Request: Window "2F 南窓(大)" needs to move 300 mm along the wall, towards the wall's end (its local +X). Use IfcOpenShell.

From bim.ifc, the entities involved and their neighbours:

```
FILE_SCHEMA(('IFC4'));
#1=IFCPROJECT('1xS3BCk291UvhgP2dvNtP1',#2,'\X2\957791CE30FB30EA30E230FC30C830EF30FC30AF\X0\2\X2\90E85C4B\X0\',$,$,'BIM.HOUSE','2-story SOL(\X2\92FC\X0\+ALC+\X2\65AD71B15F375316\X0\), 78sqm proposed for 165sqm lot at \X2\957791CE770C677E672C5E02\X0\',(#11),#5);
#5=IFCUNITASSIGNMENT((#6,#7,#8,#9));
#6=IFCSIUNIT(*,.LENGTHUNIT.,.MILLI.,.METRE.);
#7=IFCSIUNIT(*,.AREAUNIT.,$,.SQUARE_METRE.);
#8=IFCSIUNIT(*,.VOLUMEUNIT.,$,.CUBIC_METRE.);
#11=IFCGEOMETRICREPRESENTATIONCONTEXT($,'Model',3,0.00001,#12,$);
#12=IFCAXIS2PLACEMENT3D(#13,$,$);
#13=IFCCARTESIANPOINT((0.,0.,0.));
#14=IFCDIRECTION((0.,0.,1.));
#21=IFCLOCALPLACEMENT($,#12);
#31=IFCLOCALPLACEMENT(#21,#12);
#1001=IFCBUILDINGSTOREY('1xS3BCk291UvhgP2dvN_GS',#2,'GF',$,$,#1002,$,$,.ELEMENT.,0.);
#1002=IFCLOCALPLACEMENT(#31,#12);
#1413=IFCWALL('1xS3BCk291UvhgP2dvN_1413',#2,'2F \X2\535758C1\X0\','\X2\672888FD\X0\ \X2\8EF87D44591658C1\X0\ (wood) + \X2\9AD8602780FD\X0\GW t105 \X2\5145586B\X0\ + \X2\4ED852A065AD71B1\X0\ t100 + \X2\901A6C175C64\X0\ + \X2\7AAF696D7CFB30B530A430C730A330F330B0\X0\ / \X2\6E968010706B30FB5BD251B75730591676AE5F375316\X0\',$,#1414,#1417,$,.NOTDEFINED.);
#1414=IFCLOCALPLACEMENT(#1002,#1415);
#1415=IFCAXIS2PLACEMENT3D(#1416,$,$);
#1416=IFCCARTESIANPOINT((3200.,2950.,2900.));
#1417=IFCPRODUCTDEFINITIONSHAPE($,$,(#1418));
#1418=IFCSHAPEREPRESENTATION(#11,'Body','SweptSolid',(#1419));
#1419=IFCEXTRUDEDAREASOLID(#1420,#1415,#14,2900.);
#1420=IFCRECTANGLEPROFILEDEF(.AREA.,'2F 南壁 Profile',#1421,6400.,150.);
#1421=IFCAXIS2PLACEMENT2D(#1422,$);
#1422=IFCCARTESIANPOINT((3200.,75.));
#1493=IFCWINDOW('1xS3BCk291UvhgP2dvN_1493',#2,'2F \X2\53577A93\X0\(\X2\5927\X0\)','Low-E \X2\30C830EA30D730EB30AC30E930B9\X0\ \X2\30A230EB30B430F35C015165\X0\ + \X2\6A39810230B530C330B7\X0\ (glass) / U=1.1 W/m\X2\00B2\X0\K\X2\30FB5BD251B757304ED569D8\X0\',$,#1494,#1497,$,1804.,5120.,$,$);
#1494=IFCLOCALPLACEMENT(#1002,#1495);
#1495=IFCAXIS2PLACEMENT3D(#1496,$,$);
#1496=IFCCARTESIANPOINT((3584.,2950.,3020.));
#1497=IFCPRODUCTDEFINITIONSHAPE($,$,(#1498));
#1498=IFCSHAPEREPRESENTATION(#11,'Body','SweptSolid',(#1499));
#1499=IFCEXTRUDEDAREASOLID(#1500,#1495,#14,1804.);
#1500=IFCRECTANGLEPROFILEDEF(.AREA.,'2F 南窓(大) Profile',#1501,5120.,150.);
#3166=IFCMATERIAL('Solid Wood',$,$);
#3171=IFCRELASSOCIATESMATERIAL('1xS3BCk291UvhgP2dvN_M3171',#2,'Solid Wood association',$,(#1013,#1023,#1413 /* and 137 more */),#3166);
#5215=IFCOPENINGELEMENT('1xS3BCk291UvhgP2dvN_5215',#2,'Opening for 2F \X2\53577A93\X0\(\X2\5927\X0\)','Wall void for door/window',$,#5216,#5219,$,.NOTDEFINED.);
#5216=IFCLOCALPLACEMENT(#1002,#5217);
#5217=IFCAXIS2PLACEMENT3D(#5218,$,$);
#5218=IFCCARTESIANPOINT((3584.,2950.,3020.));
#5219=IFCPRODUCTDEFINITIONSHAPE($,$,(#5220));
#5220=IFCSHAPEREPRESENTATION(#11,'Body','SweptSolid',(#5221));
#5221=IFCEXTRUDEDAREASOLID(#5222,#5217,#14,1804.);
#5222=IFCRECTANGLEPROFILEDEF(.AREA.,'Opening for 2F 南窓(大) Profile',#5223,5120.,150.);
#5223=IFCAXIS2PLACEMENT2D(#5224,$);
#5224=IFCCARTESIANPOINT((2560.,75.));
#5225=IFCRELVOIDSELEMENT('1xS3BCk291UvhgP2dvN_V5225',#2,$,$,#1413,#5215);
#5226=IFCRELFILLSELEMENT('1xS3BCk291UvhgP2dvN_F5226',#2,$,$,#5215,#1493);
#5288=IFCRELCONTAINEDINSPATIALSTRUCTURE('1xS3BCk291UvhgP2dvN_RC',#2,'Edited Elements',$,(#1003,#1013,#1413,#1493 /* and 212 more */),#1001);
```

```python
import ifcopenshell
import ifcopenshell.api.geometry
import ifcopenshell.util.placement
import ifcopenshell.util.unit

model = ifcopenshell.open("bim.ifc")
unit_scale = ifcopenshell.util.unit.calculate_unit_scale(model)

window = model.by_id(1493)
opening = window.FillsVoids[0].RelatingOpeningElement
wall = opening.VoidsElements[0].RelatingBuildingElement

wall_matrix = ifcopenshell.util.placement.get_local_placement(wall.ObjectPlacement)
shift = wall_matrix[:3, 0] * 0.3 / unit_scale
before = ifcopenshell.util.placement.get_local_placement(window.ObjectPlacement)[:3, 3].copy()

# The window is not placed relative to its opening, so move both.
for product in (opening, window):
    matrix = ifcopenshell.util.placement.get_local_placement(product.ObjectPlacement)
    matrix[:3, 3] += shift
    ifcopenshell.api.geometry.edit_object_placement(model, product=product, matrix=matrix, is_si=False)

after = ifcopenshell.util.placement.get_local_placement(window.ObjectPlacement)[:3, 3]
print("window moved by", (after - before).round(3) + 0.0)

model.write("bim-out.ifc")
```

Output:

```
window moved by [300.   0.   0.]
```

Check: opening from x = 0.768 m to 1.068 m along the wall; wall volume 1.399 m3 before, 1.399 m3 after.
